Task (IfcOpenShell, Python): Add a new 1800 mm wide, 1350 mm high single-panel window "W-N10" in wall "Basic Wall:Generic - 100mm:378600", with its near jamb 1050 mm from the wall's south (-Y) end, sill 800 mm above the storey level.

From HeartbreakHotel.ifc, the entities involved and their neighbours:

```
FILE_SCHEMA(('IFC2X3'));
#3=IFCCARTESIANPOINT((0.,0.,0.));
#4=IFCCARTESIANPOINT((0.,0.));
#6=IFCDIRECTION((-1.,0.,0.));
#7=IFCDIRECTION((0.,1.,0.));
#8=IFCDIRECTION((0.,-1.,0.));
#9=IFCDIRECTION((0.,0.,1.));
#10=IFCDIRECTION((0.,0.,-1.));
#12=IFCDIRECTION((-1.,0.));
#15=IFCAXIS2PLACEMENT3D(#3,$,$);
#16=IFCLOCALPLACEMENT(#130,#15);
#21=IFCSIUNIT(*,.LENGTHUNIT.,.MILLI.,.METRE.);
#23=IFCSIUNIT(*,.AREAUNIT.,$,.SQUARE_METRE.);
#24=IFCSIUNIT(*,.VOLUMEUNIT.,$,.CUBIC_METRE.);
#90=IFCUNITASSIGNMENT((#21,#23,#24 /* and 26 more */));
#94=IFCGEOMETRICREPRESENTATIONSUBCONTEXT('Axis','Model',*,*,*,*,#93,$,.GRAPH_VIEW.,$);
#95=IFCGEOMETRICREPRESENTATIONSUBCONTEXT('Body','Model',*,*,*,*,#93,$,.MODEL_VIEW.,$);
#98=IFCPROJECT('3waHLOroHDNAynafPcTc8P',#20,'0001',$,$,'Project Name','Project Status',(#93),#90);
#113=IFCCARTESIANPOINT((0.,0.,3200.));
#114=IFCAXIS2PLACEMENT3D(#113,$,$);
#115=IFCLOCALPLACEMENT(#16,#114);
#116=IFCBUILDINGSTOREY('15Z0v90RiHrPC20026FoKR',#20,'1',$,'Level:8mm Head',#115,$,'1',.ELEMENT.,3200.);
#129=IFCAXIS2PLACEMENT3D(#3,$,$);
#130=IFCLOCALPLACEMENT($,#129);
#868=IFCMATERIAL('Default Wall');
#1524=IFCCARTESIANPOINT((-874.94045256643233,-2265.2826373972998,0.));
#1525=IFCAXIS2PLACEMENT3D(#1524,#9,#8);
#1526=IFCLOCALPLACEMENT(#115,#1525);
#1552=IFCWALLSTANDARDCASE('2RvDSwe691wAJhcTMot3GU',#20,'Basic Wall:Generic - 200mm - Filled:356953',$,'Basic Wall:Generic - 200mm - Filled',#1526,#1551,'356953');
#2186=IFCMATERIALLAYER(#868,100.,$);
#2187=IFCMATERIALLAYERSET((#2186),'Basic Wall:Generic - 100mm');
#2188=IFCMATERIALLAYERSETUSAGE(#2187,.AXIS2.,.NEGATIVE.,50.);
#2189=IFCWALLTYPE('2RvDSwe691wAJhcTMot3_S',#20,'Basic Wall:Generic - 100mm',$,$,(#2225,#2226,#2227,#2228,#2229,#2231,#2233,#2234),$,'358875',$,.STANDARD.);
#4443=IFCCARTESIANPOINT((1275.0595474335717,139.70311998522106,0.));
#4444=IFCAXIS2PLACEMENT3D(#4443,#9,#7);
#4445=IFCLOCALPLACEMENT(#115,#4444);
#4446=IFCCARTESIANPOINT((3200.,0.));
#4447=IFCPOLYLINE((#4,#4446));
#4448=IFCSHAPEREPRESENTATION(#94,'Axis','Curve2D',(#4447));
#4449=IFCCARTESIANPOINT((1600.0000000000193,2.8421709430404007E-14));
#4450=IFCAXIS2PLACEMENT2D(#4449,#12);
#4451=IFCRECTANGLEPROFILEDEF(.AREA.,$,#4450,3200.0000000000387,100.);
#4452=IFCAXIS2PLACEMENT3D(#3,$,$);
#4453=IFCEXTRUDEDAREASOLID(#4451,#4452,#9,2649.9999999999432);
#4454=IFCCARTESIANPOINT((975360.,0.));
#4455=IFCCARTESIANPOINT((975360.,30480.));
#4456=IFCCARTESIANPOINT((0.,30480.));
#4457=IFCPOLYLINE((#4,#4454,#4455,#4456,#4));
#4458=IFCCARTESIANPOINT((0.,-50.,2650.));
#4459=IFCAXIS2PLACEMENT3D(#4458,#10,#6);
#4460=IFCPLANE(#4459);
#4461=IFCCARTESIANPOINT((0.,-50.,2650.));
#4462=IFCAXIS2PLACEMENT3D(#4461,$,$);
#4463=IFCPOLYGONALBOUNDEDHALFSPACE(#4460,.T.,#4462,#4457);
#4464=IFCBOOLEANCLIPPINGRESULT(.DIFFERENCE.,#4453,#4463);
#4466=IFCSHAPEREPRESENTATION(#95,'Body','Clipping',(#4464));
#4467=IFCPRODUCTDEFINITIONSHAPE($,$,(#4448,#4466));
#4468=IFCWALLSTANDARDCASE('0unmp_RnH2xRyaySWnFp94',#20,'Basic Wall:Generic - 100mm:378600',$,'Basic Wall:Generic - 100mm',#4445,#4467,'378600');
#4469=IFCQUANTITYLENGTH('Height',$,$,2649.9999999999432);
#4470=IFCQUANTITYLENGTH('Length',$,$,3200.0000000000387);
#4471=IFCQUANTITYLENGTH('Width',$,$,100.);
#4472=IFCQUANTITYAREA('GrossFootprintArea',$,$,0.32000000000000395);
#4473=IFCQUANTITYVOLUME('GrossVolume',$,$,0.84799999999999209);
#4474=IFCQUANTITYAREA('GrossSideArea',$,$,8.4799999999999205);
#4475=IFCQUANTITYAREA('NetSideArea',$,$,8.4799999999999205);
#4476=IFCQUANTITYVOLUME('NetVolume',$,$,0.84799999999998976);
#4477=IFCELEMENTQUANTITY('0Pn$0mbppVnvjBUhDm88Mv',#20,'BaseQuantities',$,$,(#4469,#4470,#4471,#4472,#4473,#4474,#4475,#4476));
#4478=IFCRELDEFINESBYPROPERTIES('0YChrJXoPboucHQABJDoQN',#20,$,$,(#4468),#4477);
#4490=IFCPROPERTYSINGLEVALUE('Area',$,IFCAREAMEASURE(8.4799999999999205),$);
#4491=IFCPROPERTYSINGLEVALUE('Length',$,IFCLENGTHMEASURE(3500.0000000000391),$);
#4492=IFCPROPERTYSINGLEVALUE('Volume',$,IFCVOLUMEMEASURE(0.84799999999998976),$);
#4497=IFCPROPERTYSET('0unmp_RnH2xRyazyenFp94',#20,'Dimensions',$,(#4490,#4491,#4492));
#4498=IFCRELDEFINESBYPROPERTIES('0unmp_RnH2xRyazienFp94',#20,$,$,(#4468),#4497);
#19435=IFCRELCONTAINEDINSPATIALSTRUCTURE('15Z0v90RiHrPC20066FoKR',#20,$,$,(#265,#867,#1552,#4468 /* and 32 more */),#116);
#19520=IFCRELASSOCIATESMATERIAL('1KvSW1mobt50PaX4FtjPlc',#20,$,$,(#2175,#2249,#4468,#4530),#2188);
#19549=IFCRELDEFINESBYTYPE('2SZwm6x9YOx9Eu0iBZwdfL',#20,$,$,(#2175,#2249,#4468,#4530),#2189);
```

```python
import numpy as np
import ifcopenshell
import ifcopenshell.api.feature
import ifcopenshell.api.geometry
import ifcopenshell.api.pset
import ifcopenshell.api.root
import ifcopenshell.api.spatial
import ifcopenshell.api.type
import ifcopenshell.geom
import ifcopenshell.util.element
import ifcopenshell.util.placement
import ifcopenshell.util.representation
import ifcopenshell.util.shape
import ifcopenshell.util.unit

model = ifcopenshell.open("HeartbreakHotel.ifc")
unit_scale = ifcopenshell.util.unit.calculate_unit_scale(model)
area_scale = ifcopenshell.util.unit.calculate_unit_scale(model, "AREAUNIT")
volume_scale = ifcopenshell.util.unit.calculate_unit_scale(model, "VOLUMEUNIT")
settings = ifcopenshell.geom.settings()


def volume(element):
    """Net volume in cubic metres, openings subtracted."""
    shape = ifcopenshell.geom.create_shape(settings, element)
    return ifcopenshell.util.shape.get_volume(shape.geometry)


wall = model.by_guid("0unmp_RnH2xRyaySWnFp94")
storey = ifcopenshell.util.element.get_container(wall, ifc_class="IfcBuildingStorey")
context = ifcopenshell.util.representation.get_context(model, "Model", "Body", "MODEL_VIEW")
before = volume(wall)

width, height, from_end, sill = 1.8, 1.35, 1.05, 0.8  # metres

# The wall runs along its own X axis, and the end named is its -X end.
wall_shape = ifcopenshell.geom.create_shape(settings, wall)
x, y, z = ifcopenshell.util.shape.get_vertices(wall_shape.geometry).T
start = x.min() + from_end
face, thickness = float(y.min()), float(y.max() - y.min())
wall_matrix = ifcopenshell.util.placement.get_local_placement(wall.ObjectPlacement)
level = ifcopenshell.util.placement.get_local_placement(storey.ObjectPlacement)[2, 3]


def in_wall(x, y):
    """Placement at x, y metres in the wall's axes, at sill height."""
    matrix = wall_matrix.copy()
    matrix[:, 3] = wall_matrix @ np.array([x / unit_scale, y / unit_scale, 0.0, 1.0])
    matrix[2, 3] = level + sill / unit_scale
    return matrix


# Opening: a box that overshoots both wall faces by 50 mm.
opening = ifcopenshell.api.root.create_entity(model, ifc_class="IfcOpeningElement")
box = ifcopenshell.api.geometry.add_wall_representation(
    model, context=context, length=width, height=height, thickness=thickness + 0.1
)
ifcopenshell.api.geometry.assign_representation(model, product=opening, representation=box)
ifcopenshell.api.geometry.edit_object_placement(model, product=opening, matrix=in_wall(start, face - 0.05), is_si=False)
ifcopenshell.api.feature.add_feature(model, feature=opening, element=wall)

window = ifcopenshell.api.root.create_entity(model, ifc_class="IfcWindow", name="W-N10")
window.OverallWidth, window.OverallHeight = width / unit_scale, height / unit_scale
body = ifcopenshell.api.geometry.add_window_representation(
    model,
    context=context,
    overall_width=window.OverallWidth,
    overall_height=window.OverallHeight,
    partition_type="SINGLE_PANEL",
)
ifcopenshell.api.geometry.assign_representation(model, product=window, representation=body)
ifcopenshell.api.spatial.assign_container(model, products=[window], relating_structure=storey)
fills = ifcopenshell.api.feature.add_filling(model, opening=opening, element=window)
fills.OwnerHistory = window.OwnerHistory  # required in IFC2X3

# IFC2X3 keeps the operation on the window style.
style = ifcopenshell.api.root.create_entity(model, ifc_class="IfcWindowStyle", name="W-N10")
style.OperationType, style.ConstructionType = "SINGLE_PANEL", "NOTDEFINED"
style.ParameterTakesPrecedence = style.Sizeable = False
ifcopenshell.api.type.assign_type(model, related_objects=[window], relating_type=style)

# Centre the window in the wall's thickness.
ifcopenshell.api.geometry.edit_object_placement(model, product=window, matrix=in_wall(start, face), is_si=False)
window_shape = ifcopenshell.geom.create_shape(settings, window)
depth = ifcopenshell.util.shape.get_vertices(window_shape.geometry)[:, 1]
offset = face + thickness / 2 - (depth.min() + depth.max()) / 2
ifcopenshell.api.geometry.edit_object_placement(model, product=window, matrix=in_wall(start, offset), is_si=False)

after = volume(wall)

# Update the wall's stored quantities.
qto = model.by_id(ifcopenshell.util.element.get_pset(wall, "BaseQuantities", should_inherit=False)["id"])
ifcopenshell.api.pset.edit_qto(model, qto=qto, properties={
    "NetSideArea": after / thickness / area_scale,
    "NetVolume": after / volume_scale,
})
pset = model.by_id(ifcopenshell.util.element.get_pset(wall, "Dimensions", should_inherit=False)["id"])
ifcopenshell.api.pset.edit_pset(model, pset=pset, properties={
    "Area": model.create_entity("IfcAreaMeasure", after / thickness / area_scale),
    "Volume": model.create_entity("IfcVolumeMeasure", after / volume_scale),
})

print(f"wall volume {before:.3f} -> {after:.3f} m3")

model.write("HeartbreakHotel_v2.ifc")
```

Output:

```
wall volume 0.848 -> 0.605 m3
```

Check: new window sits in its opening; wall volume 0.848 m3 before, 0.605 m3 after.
